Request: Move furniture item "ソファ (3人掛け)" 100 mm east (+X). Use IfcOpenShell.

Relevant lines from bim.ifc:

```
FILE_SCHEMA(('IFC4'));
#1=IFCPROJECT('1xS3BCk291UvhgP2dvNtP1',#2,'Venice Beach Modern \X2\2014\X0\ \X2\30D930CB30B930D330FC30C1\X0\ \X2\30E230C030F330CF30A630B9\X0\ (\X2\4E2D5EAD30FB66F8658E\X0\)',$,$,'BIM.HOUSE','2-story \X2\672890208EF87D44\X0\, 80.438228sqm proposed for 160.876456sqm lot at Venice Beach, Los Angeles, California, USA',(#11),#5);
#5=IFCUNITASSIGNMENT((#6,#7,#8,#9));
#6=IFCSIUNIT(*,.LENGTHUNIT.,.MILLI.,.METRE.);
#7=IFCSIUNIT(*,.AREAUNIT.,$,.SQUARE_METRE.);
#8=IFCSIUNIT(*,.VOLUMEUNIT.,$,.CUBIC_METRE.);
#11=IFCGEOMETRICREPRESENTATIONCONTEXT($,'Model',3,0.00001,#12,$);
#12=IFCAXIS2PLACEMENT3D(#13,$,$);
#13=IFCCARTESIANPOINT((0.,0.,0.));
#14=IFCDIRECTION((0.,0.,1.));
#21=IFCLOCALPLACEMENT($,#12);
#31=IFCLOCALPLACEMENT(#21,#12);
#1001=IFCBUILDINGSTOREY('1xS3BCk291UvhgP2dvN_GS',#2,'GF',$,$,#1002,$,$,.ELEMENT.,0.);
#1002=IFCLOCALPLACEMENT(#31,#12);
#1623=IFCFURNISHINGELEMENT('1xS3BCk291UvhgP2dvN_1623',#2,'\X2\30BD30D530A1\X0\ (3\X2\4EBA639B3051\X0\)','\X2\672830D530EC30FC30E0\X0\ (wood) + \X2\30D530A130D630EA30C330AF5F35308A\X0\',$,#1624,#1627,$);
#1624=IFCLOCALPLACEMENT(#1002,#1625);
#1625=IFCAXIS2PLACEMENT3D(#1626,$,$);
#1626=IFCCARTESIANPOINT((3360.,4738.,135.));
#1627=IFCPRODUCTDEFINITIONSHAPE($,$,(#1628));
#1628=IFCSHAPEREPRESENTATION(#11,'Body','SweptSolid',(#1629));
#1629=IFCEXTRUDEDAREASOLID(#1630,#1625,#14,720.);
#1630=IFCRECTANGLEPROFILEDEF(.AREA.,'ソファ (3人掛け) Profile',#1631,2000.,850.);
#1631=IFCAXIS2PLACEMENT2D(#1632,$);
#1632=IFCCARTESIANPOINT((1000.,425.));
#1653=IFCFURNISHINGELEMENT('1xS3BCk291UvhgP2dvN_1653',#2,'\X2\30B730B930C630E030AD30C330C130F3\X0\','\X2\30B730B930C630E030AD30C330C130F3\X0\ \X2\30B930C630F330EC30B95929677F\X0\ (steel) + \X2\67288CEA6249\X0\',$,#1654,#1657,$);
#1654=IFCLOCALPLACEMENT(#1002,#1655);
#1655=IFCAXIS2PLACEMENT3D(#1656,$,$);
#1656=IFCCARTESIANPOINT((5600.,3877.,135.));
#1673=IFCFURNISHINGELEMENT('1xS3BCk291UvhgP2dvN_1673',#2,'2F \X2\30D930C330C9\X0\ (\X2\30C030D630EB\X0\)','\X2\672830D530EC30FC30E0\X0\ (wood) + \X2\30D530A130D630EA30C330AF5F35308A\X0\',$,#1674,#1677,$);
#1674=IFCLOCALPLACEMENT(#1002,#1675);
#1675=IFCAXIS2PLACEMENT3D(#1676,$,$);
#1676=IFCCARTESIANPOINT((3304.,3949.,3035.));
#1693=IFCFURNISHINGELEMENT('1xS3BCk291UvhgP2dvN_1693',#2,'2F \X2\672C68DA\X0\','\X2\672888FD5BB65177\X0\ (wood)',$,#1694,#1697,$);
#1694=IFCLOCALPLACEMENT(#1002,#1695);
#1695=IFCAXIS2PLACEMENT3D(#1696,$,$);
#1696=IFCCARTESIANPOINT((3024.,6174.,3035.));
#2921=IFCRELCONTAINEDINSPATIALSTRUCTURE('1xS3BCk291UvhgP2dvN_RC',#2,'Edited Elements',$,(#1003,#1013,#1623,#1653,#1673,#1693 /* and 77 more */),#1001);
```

```python
import ifcopenshell
import ifcopenshell.api.geometry
import ifcopenshell.util.placement

model = ifcopenshell.open("bim.ifc")

item = model.by_guid("1xS3BCk291UvhgP2dvN_1623")
matrix = ifcopenshell.util.placement.get_local_placement(item.ObjectPlacement)
matrix[0, 3] += 100.0
ifcopenshell.api.geometry.edit_object_placement(model, product=item, matrix=matrix, is_si=False)

print(ifcopenshell.util.placement.get_local_placement(item.ObjectPlacement).round(3) + 0.0)

model.write("bim-out.ifc")
```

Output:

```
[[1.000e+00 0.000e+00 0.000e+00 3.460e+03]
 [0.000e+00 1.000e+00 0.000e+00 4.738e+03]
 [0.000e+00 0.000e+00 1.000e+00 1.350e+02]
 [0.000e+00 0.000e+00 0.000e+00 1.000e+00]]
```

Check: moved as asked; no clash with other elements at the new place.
